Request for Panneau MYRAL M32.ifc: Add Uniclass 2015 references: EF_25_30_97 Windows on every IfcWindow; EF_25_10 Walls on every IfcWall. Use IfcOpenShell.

First a look at what the model holds.

```python
import ifcopenshell

model = ifcopenshell.open("Panneau MYRAL M32.ifc")
print(model.schema)
print("classifications:", [c.Name for c in model.by_type("IfcClassification")])
for ifc_class in ("IfcDoor", "IfcRoof", "IfcStair", "IfcWall", "IfcWindow"):
    print(ifc_class, len(model.by_type(ifc_class)))
```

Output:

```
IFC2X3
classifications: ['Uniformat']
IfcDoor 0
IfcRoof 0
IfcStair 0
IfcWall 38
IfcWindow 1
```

```python
import ifcopenshell
import ifcopenshell.api.classification

model = ifcopenshell.open("Panneau MYRAL M32.ifc")

# IFC2X3 requires Source and Edition and has no link from the project to the system.
system = model.create_entity("IfcClassification", Source="NBS", Edition="2015", Name="Uniclass 2015")

codes = {
    "IfcWindow": ("EF_25_30_97", "Windows"),
    "IfcWall": ("EF_25_10", "Walls"),
}
for ifc_class, (code, name) in codes.items():
    products = model.by_type(ifc_class)
    ifcopenshell.api.classification.add_reference(
        model, products=products, classification=system, identification=code, name=name
    )
    print(code, len(products))

model.write("Panneau MYRAL M32_v2.ifc")
```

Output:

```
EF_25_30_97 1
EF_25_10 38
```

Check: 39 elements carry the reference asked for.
